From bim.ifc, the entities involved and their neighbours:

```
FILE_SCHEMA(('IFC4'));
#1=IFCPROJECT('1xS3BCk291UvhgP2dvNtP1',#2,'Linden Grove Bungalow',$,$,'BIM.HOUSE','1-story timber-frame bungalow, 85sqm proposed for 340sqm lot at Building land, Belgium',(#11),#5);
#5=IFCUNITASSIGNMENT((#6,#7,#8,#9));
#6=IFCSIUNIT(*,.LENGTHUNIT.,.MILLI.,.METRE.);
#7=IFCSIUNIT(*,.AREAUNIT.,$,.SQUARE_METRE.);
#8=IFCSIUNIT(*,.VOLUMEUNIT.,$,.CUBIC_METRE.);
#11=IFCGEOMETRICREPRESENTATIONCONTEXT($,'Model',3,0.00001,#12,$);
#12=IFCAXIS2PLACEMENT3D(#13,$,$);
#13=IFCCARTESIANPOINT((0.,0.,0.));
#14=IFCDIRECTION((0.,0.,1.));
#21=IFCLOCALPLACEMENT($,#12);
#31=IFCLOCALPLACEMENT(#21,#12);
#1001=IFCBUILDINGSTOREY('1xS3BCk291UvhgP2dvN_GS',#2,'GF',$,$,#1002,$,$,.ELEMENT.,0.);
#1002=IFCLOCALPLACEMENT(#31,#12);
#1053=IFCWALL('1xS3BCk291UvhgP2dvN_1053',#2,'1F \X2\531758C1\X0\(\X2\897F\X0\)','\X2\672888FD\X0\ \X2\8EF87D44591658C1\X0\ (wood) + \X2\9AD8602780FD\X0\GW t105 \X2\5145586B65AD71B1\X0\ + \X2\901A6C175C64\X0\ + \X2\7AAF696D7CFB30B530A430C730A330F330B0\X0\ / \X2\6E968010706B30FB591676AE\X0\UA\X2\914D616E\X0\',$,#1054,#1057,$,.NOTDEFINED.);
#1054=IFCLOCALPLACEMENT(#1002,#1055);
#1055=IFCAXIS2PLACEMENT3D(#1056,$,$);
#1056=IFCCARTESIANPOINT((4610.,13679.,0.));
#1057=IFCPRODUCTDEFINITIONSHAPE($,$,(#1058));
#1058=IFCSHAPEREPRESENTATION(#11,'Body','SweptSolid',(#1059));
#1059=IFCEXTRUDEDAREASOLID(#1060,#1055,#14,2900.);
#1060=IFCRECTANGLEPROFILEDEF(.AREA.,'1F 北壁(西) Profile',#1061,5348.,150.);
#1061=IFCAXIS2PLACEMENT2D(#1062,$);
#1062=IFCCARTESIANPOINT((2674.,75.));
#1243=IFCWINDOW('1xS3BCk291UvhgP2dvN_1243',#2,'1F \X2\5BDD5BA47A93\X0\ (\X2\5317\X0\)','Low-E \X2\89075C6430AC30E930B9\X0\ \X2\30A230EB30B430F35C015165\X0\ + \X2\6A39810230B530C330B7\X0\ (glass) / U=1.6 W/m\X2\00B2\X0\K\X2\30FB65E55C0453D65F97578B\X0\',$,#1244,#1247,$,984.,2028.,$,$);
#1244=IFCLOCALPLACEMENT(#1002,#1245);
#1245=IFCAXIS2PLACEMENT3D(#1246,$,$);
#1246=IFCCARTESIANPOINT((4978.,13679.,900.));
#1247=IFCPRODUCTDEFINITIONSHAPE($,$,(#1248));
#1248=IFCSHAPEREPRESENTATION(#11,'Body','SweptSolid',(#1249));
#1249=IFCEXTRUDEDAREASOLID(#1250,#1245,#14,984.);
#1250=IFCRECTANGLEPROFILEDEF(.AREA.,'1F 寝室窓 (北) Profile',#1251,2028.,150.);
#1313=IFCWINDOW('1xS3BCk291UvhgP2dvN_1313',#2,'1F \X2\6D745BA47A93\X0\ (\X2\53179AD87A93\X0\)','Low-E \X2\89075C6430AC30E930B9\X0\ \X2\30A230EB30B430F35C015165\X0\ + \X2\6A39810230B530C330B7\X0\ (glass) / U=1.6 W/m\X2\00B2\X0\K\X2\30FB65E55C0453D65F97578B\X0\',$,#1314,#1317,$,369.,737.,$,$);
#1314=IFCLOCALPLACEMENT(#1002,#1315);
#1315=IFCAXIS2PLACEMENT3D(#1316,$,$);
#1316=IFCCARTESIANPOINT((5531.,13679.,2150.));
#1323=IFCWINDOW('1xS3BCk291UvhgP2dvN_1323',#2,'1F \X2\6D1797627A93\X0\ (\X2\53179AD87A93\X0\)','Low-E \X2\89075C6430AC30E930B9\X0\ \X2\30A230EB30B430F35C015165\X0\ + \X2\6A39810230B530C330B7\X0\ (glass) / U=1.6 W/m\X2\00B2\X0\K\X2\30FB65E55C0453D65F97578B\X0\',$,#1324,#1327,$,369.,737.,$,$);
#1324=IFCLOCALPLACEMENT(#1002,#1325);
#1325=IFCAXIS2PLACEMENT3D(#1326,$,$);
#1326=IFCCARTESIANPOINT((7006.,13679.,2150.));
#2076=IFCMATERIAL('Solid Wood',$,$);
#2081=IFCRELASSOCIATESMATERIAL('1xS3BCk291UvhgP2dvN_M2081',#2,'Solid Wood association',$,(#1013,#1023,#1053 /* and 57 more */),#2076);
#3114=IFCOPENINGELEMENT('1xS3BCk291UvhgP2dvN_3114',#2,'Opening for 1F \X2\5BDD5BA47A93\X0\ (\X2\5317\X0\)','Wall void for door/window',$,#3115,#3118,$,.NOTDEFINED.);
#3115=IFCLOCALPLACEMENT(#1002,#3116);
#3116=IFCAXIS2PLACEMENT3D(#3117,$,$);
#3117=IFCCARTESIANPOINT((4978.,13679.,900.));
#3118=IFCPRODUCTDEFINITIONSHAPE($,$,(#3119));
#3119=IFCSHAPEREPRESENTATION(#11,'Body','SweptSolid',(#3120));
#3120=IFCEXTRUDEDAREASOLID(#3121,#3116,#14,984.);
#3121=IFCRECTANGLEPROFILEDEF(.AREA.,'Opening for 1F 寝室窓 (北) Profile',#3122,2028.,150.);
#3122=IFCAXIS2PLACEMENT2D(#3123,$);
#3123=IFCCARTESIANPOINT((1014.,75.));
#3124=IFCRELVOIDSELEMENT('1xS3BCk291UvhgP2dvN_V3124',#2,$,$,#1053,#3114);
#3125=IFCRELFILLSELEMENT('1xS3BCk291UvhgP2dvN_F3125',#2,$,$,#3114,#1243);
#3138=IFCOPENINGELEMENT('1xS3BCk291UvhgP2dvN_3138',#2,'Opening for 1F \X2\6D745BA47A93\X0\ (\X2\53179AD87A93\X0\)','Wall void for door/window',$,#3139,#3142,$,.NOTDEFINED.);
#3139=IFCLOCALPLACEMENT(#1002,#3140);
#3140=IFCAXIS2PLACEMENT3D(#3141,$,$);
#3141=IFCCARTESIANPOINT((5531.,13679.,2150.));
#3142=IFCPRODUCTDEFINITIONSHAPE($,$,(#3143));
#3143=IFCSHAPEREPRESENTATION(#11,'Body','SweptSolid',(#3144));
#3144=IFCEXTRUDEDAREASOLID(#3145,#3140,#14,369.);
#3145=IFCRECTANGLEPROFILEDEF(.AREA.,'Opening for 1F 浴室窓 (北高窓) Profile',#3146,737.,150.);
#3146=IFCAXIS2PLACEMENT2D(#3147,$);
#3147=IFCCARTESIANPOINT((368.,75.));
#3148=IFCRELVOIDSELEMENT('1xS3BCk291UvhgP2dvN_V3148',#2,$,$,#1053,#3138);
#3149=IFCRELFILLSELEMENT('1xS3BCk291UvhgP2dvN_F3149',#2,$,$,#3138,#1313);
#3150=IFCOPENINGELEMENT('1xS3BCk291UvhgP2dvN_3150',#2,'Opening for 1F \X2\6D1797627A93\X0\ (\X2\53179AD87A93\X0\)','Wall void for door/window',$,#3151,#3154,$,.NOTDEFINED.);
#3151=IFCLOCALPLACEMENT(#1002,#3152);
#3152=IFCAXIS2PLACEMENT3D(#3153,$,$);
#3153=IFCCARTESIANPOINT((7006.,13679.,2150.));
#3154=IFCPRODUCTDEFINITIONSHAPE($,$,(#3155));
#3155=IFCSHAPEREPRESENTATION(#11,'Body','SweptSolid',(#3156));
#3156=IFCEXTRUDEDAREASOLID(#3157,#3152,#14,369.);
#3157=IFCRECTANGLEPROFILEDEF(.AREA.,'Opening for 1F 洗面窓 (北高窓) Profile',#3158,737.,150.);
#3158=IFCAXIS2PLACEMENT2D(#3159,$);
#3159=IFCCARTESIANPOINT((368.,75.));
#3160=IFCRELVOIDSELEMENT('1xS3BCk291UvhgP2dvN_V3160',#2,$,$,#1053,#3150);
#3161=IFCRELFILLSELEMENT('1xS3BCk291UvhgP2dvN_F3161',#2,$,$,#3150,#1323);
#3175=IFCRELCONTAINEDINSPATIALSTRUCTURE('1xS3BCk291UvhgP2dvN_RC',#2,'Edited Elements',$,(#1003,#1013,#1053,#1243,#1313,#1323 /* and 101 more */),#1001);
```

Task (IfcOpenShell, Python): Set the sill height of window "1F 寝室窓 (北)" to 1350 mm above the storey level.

```python
import numpy as np
import ifcopenshell
import ifcopenshell.api.geometry
import ifcopenshell.geom
import ifcopenshell.util.element
import ifcopenshell.util.placement
import ifcopenshell.util.shape
import ifcopenshell.util.unit

model = ifcopenshell.open("bim.ifc")
unit_scale = ifcopenshell.util.unit.calculate_unit_scale(model)

window = model.by_id(1243)
opening = window.FillsVoids[0].RelatingOpeningElement
storey = ifcopenshell.util.element.get_container(window, ifc_class="IfcBuildingStorey")
level = ifcopenshell.util.placement.get_local_placement(storey.ObjectPlacement)[2, 3]

# The opening's origin need not be at the sill, so measure its lowest point.
shape = ifcopenshell.geom.create_shape(ifcopenshell.geom.settings(), opening)
bottom = ifcopenshell.util.shape.get_shape_bottom_elevation(shape, shape.geometry) / unit_scale
dz = level + 1.35 / unit_scale - bottom

shift = np.array([0.0, 0.0, dz])
# The window is not placed relative to its opening, so move both.
for product in (opening, window):
    matrix = ifcopenshell.util.placement.get_local_placement(product.ObjectPlacement)
    matrix[:3, 3] += shift
    ifcopenshell.api.geometry.edit_object_placement(model, product=product, matrix=matrix, is_si=False)

print(f"moved by {dz * unit_scale:+.3f} m")

model.write("bim_updated.ifc")
```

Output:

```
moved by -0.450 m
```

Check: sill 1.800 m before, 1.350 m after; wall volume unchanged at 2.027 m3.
